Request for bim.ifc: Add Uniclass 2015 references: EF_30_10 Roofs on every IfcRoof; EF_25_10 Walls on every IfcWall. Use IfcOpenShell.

First a look at what the model holds.

```python
import ifcopenshell

model = ifcopenshell.open("bim.ifc")
print(model.schema)
print("classifications:", [c.Name for c in model.by_type("IfcClassification")])
for ifc_class in ("IfcDoor", "IfcRoof", "IfcStair", "IfcWall", "IfcWindow"):
    print(ifc_class, len(model.by_type(ifc_class)))
```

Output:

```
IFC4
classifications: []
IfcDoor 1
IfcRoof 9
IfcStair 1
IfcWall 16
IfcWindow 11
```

```python
import ifcopenshell
import ifcopenshell.api.classification

model = ifcopenshell.open("bim.ifc")

system = ifcopenshell.api.classification.add_classification(model, classification="Uniclass 2015")

codes = {
    "IfcRoof": ("EF_30_10", "Roofs"),
    "IfcWall": ("EF_25_10", "Walls"),
}
for ifc_class, (code, name) in codes.items():
    products = model.by_type(ifc_class)
    ifcopenshell.api.classification.add_reference(
        model, products=products, classification=system, identification=code, name=name
    )
    print(code, len(products))

model.write("bim_updated.ifc")
```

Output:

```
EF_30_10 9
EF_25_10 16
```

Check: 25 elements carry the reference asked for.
